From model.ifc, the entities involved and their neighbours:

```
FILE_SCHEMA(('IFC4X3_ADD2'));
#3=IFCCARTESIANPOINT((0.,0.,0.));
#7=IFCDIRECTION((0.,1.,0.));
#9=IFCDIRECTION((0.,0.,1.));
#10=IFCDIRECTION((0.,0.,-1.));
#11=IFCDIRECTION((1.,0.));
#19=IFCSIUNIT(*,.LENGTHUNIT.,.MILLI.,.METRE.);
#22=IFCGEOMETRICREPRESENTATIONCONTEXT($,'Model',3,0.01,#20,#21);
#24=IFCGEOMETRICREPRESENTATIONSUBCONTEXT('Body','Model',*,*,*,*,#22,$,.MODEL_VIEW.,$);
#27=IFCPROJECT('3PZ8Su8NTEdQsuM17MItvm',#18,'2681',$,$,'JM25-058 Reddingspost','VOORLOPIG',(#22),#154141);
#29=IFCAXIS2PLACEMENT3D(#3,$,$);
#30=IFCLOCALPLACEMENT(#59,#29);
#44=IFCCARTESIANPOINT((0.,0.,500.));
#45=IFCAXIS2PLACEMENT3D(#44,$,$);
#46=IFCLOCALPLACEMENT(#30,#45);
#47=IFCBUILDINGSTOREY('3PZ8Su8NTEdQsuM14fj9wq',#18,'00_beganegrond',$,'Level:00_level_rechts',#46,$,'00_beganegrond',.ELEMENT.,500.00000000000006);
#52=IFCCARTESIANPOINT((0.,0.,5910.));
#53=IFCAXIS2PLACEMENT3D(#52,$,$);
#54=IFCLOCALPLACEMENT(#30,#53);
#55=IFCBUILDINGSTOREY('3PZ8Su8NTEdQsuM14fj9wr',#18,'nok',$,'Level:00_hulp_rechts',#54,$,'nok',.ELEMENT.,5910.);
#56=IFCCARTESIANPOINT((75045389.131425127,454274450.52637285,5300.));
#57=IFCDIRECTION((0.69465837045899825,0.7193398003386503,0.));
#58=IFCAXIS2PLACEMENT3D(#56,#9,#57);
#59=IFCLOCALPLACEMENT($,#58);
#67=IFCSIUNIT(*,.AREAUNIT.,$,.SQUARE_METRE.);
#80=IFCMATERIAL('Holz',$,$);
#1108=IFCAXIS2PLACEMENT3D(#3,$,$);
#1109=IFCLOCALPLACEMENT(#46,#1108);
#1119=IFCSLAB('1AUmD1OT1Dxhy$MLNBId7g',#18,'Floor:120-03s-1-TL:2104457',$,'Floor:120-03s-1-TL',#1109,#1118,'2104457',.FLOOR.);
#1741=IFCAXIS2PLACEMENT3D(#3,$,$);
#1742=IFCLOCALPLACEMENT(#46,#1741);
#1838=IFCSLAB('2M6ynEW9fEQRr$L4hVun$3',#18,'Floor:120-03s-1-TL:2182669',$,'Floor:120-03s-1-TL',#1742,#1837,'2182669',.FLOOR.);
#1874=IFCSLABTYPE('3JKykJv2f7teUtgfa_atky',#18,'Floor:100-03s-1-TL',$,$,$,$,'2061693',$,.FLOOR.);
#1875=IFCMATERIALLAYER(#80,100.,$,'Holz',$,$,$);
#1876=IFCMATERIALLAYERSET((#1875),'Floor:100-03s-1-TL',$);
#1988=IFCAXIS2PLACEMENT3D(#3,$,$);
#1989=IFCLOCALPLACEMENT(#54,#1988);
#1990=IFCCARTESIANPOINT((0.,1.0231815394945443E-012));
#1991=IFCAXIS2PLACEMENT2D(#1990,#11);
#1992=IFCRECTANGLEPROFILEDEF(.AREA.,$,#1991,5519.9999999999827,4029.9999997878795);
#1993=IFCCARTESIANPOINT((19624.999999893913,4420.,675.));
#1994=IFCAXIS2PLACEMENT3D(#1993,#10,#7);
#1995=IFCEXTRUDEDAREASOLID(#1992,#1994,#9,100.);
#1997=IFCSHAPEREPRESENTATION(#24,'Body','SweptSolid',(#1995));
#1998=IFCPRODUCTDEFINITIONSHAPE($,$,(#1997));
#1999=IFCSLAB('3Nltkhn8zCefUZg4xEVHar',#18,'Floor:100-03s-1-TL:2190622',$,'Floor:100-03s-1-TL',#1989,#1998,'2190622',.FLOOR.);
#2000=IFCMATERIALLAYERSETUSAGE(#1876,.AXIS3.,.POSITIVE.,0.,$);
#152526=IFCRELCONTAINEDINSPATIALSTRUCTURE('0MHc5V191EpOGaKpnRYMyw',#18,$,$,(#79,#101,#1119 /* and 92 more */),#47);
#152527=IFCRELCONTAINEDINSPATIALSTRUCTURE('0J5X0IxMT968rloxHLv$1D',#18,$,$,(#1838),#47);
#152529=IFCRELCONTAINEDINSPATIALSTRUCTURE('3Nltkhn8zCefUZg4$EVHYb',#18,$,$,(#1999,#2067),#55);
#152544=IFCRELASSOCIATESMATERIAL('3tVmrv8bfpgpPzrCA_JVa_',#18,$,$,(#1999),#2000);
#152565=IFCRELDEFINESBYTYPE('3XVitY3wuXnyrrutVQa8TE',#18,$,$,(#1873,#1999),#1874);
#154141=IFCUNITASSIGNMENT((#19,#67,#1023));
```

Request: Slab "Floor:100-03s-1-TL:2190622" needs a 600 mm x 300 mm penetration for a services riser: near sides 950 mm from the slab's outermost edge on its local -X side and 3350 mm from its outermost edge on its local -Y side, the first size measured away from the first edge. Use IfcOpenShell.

```python
import numpy as np
import ifcopenshell
import ifcopenshell.api.feature
import ifcopenshell.api.geometry
import ifcopenshell.api.root
import ifcopenshell.geom
import ifcopenshell.util.placement
import ifcopenshell.util.representation
import ifcopenshell.util.shape
import ifcopenshell.util.unit

model = ifcopenshell.open("model.ifc")
unit_scale = ifcopenshell.util.unit.calculate_unit_scale(model)
settings = ifcopenshell.geom.settings()


def volume(element):
    """Net volume in cubic metres, openings subtracted."""
    shape = ifcopenshell.geom.create_shape(settings, element)
    return ifcopenshell.util.shape.get_volume(shape.geometry)


slab = model.by_guid("3Nltkhn8zCefUZg4xEVHar")
before = volume(slab)

# Extent in the slab's own axes, in metres. The edges named are its -X and -Y sides.
slab_shape = ifcopenshell.geom.create_shape(settings, slab)
vertices = ifcopenshell.util.shape.get_vertices(slab_shape.geometry)
x_min, y_min, bottom = vertices.min(axis=0)
top = vertices[:, 2].max()

opening = ifcopenshell.api.root.create_entity(model, ifc_class="IfcOpeningElement", name="Services riser opening", predefined_type="OPENING")
context = ifcopenshell.util.representation.get_context(model, "Model", "Body", "MODEL_VIEW")
width, depth = 0.6, 0.3
outline = [(0.0, 0.0), (width, 0.0), (width, depth), (0.0, depth), (0.0, 0.0)]
# Overshoot both faces by 50 mm so the cut is clean.
shape = ifcopenshell.api.geometry.add_slab_representation(
    model, context=context, depth=top - bottom + 0.1, polyline=outline
)
ifcopenshell.api.geometry.assign_representation(model, product=opening, representation=shape)

matrix = ifcopenshell.util.placement.get_local_placement(slab.ObjectPlacement)
matrix[:, 3] = matrix @ np.append(np.array([x_min + 0.95, y_min + 3.35, bottom - 0.05]) / unit_scale, 1.0)
ifcopenshell.api.geometry.edit_object_placement(model, product=opening, matrix=matrix, is_si=False)
ifcopenshell.api.feature.add_feature(model, feature=opening, element=slab)

after = volume(slab)

print(f"slab volume {before:.3f} -> {after:.3f} m3")

model.write("model_rev.ifc")
```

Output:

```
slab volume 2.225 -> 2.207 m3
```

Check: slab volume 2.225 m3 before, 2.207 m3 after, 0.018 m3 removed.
